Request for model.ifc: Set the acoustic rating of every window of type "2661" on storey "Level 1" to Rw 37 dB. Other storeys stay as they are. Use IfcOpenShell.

First a look at what the model holds.

```python
import ifcopenshell
import ifcopenshell.util.element

model = ifcopenshell.open("model.ifc")
print(model.schema)
storey = next(s for s in model.by_type("IfcBuildingStorey") if s.Name == "Level 1")
windows = [e for e in ifcopenshell.util.element.get_decomposition(storey) if e.is_a("IfcWindow")]
seen = {}
for e in windows:
    element_type = ifcopenshell.util.element.get_type(e)
    key = (element_type.Name if element_type != e and element_type else None, ifcopenshell.util.element.get_pset(e, "Pset_WindowCommon", "AcousticRating"))
    seen[key] = seen.get(key, 0) + 1
for (name, value), count in sorted(seen.items(), key=str):
    print(count, "x", name, "|", value)
```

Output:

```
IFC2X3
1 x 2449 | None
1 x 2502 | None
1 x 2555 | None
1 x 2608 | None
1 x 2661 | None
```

```python
import ifcopenshell
import ifcopenshell.api.pset
import ifcopenshell.util.element

model = ifcopenshell.open("model.ifc")

storey = next(s for s in model.by_type("IfcBuildingStorey") if s.Name == "Level 1")
windows = [e for e in ifcopenshell.util.element.get_decomposition(storey) if e.is_a("IfcWindow")]

count = 0
for e in windows:
    element_type = ifcopenshell.util.element.get_type(e)
    if element_type in (None, e) or element_type.Name != "2661":
        continue
    # add_pset returns the element's existing set when there is one.
    pset = ifcopenshell.api.pset.add_pset(model, product=e, name="Pset_WindowCommon")
    ifcopenshell.api.pset.edit_pset(model, pset=pset, properties={"AcousticRating": "Rw 37 dB"})
    count += 1

print(count, "windows updated")

model.write("model_rev.ifc")
```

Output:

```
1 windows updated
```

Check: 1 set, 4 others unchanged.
